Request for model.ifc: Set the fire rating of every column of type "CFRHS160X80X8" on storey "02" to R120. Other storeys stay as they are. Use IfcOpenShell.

First a look at what the model holds.

```python
import ifcopenshell
import ifcopenshell.util.element

model = ifcopenshell.open("model.ifc")
print(model.schema)
storey = next(s for s in model.by_type("IfcBuildingStorey") if s.Name == "02")
columns = [e for e in ifcopenshell.util.element.get_decomposition(storey) if e.is_a("IfcColumn")]
seen = {}
for e in columns:
    element_type = ifcopenshell.util.element.get_type(e)
    key = (element_type.Name if element_type != e and element_type else None, ifcopenshell.util.element.get_pset(e, "Pset_ColumnCommon", "FireRating"))
    seen[key] = seen.get(key, 0) + 1
for (name, value), count in sorted(seen.items(), key=str):
    print(count, "x", name, "|", value)
```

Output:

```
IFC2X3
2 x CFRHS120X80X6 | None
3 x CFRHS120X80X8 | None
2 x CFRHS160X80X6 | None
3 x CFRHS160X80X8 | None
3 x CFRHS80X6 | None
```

```python
import ifcopenshell
import ifcopenshell.api.pset
import ifcopenshell.util.element

model = ifcopenshell.open("model.ifc")

storey = next(s for s in model.by_type("IfcBuildingStorey") if s.Name == "02")
columns = [e for e in ifcopenshell.util.element.get_decomposition(storey) if e.is_a("IfcColumn")]

count = 0
for e in columns:
    element_type = ifcopenshell.util.element.get_type(e)
    if element_type in (None, e) or element_type.Name != "CFRHS160X80X8":
        continue
    # add_pset returns the element's existing set when there is one.
    pset = ifcopenshell.api.pset.add_pset(model, product=e, name="Pset_ColumnCommon")
    ifcopenshell.api.pset.edit_pset(model, pset=pset, properties={"FireRating": "R120"})
    count += 1

print(count, "columns updated")

model.write("model_rev.ifc")
```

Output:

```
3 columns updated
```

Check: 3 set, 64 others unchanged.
